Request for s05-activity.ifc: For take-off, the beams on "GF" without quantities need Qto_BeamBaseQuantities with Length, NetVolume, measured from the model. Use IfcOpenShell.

First a look at what the model holds.

```python
import ifcopenshell
import ifcopenshell.util.element
import ifcopenshell.util.unit

model = ifcopenshell.open("s05-activity.ifc")
print(model.schema)
for unit_type in ("LENGTHUNIT", "AREAUNIT", "VOLUMEUNIT"):
    print(unit_type, ifcopenshell.util.unit.calculate_unit_scale(model, unit_type))
storey = next(s for s in model.by_type("IfcBuildingStorey") if s.Name == "GF")
beams = [e for e in ifcopenshell.util.element.get_decomposition(storey) if e.is_a("IfcBeam")]
for e in sorted(beams, key=lambda e: e.id()):
    print(e.id(), e.is_a(), e.Name, list(ifcopenshell.util.element.get_psets(e, qtos_only=True)), sep=" | ")
```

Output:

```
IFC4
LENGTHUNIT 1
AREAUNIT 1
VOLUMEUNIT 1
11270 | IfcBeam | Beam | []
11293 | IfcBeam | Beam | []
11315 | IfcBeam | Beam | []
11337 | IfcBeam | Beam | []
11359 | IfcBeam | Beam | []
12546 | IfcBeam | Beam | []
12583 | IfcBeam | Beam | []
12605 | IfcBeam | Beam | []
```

```python
import ifcopenshell
import ifcopenshell.api.pset
import ifcopenshell.geom
import ifcopenshell.util.element
import ifcopenshell.util.shape
import ifcopenshell.util.unit

model = ifcopenshell.open("s05-activity.ifc")
unit_scale = ifcopenshell.util.unit.calculate_unit_scale(model)
volume_scale = ifcopenshell.util.unit.calculate_unit_scale(model, "VOLUMEUNIT")
settings = ifcopenshell.geom.settings()

storey = next(s for s in model.by_type("IfcBuildingStorey") if s.Name == "GF")
beams = [e for e in ifcopenshell.util.element.get_decomposition(storey) if e.is_a("IfcBeam")]

for e in sorted(beams, key=lambda e: e.id()):
    if ifcopenshell.util.element.get_psets(e, qtos_only=True, should_inherit=False):
        continue
    # Geometry comes back in metres, in the element's own axes.
    shape = ifcopenshell.geom.create_shape(settings, e)
    values = {
        "Length": ifcopenshell.util.shape.get_max_xyz(shape.geometry) / unit_scale,
        "NetVolume": ifcopenshell.util.shape.get_volume(shape.geometry) / volume_scale,
    }
    qto = ifcopenshell.api.pset.add_qto(model, product=e, name="Qto_BeamBaseQuantities")
    ifcopenshell.api.pset.edit_qto(model, qto=qto, properties=values)
    print(e.id(), {k: round(v, 3) for k, v in values.items()})

model.write("s05-activity_v2.ifc")
```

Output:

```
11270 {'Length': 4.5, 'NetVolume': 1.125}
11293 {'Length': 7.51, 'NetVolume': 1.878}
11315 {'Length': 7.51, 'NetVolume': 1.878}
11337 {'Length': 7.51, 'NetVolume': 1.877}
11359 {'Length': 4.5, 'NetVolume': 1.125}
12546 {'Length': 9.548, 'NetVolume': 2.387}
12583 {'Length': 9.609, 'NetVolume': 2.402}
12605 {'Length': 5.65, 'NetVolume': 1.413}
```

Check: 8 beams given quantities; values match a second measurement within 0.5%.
